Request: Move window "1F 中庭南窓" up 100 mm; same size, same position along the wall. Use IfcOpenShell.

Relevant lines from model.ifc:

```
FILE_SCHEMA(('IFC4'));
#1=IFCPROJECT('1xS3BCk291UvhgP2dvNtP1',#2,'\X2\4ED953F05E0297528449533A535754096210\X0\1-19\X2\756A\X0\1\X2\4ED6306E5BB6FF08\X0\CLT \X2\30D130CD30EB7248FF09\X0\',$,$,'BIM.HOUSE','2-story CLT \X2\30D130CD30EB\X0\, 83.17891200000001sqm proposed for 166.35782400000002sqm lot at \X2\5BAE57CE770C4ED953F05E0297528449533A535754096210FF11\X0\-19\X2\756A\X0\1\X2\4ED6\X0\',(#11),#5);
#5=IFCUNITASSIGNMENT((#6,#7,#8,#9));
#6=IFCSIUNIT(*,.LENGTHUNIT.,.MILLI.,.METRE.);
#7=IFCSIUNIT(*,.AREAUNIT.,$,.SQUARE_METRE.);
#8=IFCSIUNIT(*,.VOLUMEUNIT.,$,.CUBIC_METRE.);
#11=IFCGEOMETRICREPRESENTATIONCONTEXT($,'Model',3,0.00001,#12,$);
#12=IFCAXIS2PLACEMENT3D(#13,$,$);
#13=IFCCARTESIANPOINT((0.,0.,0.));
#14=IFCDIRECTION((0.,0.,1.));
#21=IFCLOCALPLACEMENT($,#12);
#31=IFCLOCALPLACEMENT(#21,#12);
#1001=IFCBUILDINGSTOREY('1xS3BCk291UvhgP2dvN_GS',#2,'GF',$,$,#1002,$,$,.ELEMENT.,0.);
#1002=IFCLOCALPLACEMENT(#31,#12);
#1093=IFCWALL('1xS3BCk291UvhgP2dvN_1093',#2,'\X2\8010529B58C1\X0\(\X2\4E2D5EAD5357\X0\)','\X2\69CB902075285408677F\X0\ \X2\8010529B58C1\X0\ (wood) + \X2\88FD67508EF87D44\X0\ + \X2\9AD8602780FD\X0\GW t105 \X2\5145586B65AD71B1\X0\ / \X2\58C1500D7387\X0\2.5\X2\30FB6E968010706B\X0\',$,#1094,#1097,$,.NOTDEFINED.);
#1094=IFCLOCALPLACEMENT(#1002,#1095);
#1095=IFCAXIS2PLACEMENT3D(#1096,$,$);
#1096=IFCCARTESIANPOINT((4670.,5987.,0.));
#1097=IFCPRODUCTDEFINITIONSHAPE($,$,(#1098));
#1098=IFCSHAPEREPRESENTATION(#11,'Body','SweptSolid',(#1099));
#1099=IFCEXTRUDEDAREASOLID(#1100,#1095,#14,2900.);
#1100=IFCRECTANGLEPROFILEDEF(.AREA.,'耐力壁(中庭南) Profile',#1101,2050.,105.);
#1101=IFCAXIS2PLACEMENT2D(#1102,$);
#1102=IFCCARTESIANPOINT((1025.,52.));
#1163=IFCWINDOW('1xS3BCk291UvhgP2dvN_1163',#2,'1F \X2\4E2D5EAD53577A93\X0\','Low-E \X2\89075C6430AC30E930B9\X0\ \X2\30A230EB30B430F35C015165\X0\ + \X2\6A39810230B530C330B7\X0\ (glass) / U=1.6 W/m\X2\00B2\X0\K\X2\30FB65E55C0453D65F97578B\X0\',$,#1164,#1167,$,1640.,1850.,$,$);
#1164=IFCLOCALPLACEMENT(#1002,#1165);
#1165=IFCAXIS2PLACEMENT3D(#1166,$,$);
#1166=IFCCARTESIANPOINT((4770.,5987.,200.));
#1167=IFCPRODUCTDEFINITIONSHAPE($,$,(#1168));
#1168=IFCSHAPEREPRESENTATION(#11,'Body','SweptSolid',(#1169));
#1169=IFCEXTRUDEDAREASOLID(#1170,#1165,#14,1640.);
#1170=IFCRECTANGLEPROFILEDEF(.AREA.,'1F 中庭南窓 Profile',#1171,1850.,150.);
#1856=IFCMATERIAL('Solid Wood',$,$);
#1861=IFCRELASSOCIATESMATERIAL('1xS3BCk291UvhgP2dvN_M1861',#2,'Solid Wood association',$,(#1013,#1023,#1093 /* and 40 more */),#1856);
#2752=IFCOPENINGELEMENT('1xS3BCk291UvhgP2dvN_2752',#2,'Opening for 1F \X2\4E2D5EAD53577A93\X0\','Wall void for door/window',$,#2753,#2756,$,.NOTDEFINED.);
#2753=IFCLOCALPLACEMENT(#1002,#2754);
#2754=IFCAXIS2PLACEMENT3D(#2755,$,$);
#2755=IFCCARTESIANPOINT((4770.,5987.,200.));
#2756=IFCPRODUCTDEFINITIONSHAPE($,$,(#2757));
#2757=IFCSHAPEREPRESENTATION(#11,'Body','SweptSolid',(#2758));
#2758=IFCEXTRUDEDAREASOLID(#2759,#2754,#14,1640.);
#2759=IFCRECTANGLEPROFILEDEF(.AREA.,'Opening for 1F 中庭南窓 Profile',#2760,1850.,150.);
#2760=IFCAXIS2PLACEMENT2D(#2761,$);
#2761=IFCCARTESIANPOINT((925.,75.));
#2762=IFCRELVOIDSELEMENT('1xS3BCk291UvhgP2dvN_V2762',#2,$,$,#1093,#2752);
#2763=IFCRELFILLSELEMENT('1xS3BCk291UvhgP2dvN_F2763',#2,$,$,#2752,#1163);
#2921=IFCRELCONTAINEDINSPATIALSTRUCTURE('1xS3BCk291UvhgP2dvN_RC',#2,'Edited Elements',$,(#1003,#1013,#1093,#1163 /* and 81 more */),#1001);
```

```python
import numpy as np
import ifcopenshell
import ifcopenshell.api.geometry
import ifcopenshell.util.placement
import ifcopenshell.util.unit

model = ifcopenshell.open("model.ifc")
unit_scale = ifcopenshell.util.unit.calculate_unit_scale(model)

window = model.by_id(1163)
opening = window.FillsVoids[0].RelatingOpeningElement
dz = 100.0

shift = np.array([0.0, 0.0, dz])
# The window is not placed relative to its opening, so move both.
for product in (opening, window):
    matrix = ifcopenshell.util.placement.get_local_placement(product.ObjectPlacement)
    matrix[:3, 3] += shift
    ifcopenshell.api.geometry.edit_object_placement(model, product=product, matrix=matrix, is_si=False)

print(f"moved by {dz * unit_scale:+.3f} m")

model.write("model_updated.ifc")
```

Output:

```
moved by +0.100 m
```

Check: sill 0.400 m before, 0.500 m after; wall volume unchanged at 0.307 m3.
